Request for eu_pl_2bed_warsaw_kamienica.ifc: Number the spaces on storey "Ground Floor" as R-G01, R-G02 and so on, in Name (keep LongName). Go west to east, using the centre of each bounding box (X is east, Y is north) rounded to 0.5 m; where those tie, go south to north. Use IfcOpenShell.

First a look at what the model holds.

```python
import ifcopenshell
import ifcopenshell.util.element
import ifcopenshell.util.placement

model = ifcopenshell.open("eu_pl_2bed_warsaw_kamienica.ifc")
print(model.schema)
storey = next(s for s in model.by_type("IfcBuildingStorey") if s.Name == "Ground Floor")
spaces = [e for e in ifcopenshell.util.element.get_decomposition(storey) if e.is_a("IfcSpace")]
for e in sorted(spaces, key=lambda e: e.id()):
    origin = ifcopenshell.util.placement.get_local_placement(e.ObjectPlacement)[:3, 3]
    print(e.id(), e.Name, e.LongName, origin.round(2) + 0.0, sep=" | ")
```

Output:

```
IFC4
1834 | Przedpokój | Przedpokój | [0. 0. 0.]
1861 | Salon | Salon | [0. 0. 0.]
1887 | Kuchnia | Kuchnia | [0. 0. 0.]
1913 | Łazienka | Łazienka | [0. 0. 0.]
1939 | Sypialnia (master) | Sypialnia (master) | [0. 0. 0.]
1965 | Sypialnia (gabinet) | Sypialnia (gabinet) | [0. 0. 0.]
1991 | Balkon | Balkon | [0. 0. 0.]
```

```python
import ifcopenshell
import ifcopenshell.geom
import ifcopenshell.util.element
import ifcopenshell.util.shape

model = ifcopenshell.open("eu_pl_2bed_warsaw_kamienica.ifc")
settings = ifcopenshell.geom.settings()
settings.set("use-world-coords", True)


def centre(element):
    shape = ifcopenshell.geom.create_shape(settings, element)
    return ifcopenshell.util.shape.get_bbox_centroid(shape.geometry)


storey = next(s for s in model.by_type("IfcBuildingStorey") if s.Name == "Ground Floor")
spaces = [e for e in ifcopenshell.util.element.get_decomposition(storey) if e.is_a("IfcSpace")]

# Insertion points can sit at a corner or the storey origin, so sort by the geometry (in metres).
centres = {e: centre(e) for e in spaces}
spaces.sort(key=lambda e: (round(centres[e][0] / 0.5), centres[e][1]))

for i, e in enumerate(spaces, start=1):
    number = f"R-G{i:02d}"
    e.Name = number
    print(e.id(), number)

model.write("eu_pl_2bed_warsaw_kamienica_edited.ifc")
```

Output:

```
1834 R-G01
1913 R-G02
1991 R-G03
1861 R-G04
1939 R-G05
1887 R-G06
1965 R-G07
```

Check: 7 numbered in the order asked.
